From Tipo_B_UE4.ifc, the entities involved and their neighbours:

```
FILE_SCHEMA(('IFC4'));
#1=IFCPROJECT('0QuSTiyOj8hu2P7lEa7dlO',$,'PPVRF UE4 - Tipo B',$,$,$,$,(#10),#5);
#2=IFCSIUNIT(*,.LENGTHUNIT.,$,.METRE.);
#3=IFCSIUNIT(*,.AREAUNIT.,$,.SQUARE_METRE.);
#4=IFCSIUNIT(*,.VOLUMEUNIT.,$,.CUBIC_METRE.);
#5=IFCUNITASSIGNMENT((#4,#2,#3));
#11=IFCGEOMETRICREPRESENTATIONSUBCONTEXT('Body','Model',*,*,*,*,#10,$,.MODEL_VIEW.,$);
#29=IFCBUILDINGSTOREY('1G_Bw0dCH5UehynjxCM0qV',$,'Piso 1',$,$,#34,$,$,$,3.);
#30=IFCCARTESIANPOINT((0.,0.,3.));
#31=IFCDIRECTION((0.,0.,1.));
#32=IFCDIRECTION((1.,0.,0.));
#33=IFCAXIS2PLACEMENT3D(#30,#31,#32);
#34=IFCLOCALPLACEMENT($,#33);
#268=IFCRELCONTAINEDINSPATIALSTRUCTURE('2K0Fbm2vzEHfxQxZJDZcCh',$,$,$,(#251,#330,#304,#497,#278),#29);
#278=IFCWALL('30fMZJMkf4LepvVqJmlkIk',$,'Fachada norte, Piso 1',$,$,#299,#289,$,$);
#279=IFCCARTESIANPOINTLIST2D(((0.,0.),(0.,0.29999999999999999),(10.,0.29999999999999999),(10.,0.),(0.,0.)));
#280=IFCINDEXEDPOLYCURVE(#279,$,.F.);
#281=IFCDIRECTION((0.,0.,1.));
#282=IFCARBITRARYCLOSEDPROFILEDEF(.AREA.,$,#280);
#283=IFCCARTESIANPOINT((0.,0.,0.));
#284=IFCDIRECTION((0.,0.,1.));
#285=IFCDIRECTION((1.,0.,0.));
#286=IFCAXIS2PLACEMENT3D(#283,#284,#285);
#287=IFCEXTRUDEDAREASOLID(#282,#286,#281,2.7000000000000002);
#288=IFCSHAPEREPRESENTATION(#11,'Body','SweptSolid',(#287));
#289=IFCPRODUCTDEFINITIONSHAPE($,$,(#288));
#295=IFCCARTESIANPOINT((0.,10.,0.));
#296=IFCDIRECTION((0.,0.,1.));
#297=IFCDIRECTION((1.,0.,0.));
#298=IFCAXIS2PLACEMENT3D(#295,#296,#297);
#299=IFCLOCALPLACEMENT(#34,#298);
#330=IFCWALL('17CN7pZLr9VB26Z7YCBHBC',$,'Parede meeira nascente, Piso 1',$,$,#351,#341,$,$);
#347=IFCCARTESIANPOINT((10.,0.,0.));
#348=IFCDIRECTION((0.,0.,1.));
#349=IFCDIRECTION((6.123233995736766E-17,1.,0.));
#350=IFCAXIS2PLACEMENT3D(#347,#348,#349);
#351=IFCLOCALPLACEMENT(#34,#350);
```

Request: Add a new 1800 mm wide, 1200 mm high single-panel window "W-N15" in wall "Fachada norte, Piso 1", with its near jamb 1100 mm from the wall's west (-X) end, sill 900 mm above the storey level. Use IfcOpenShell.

```python
import numpy as np
import ifcopenshell
import ifcopenshell.api.feature
import ifcopenshell.api.geometry
import ifcopenshell.api.root
import ifcopenshell.api.spatial
import ifcopenshell.geom
import ifcopenshell.util.element
import ifcopenshell.util.placement
import ifcopenshell.util.representation
import ifcopenshell.util.shape
import ifcopenshell.util.unit

model = ifcopenshell.open("Tipo_B_UE4.ifc")
unit_scale = ifcopenshell.util.unit.calculate_unit_scale(model)
settings = ifcopenshell.geom.settings()


def volume(element):
    """Net volume in cubic metres, openings subtracted."""
    shape = ifcopenshell.geom.create_shape(settings, element)
    return ifcopenshell.util.shape.get_volume(shape.geometry)


wall = model.by_id(278)
storey = ifcopenshell.util.element.get_container(wall, ifc_class="IfcBuildingStorey")
context = ifcopenshell.util.representation.get_context(model, "Model", "Body", "MODEL_VIEW")
before = volume(wall)

width, height, from_end, sill = 1.8, 1.2, 1.1, 0.9  # metres

# The wall runs along its own X axis, and the end named is its -X end.
wall_shape = ifcopenshell.geom.create_shape(settings, wall)
x, y, z = ifcopenshell.util.shape.get_vertices(wall_shape.geometry).T
start = x.min() + from_end
face, thickness = float(y.min()), float(y.max() - y.min())
wall_matrix = ifcopenshell.util.placement.get_local_placement(wall.ObjectPlacement)
level = ifcopenshell.util.placement.get_local_placement(storey.ObjectPlacement)[2, 3]


def in_wall(x, y):
    """Placement at x, y metres in the wall's axes, at sill height."""
    matrix = wall_matrix.copy()
    matrix[:, 3] = wall_matrix @ np.array([x / unit_scale, y / unit_scale, 0.0, 1.0])
    matrix[2, 3] = level + sill / unit_scale
    return matrix


# Opening: a box that overshoots both wall faces by 50 mm.
opening = ifcopenshell.api.root.create_entity(model, ifc_class="IfcOpeningElement", predefined_type="OPENING")
box = ifcopenshell.api.geometry.add_wall_representation(
    model, context=context, length=width, height=height, thickness=thickness + 0.1
)
ifcopenshell.api.geometry.assign_representation(model, product=opening, representation=box)
ifcopenshell.api.geometry.edit_object_placement(model, product=opening, matrix=in_wall(start, face - 0.05), is_si=False)
ifcopenshell.api.feature.add_feature(model, feature=opening, element=wall)

window = ifcopenshell.api.root.create_entity(model, ifc_class="IfcWindow", name="W-N15", predefined_type="WINDOW")
window.OverallWidth, window.OverallHeight = width / unit_scale, height / unit_scale
window.PartitioningType = "SINGLE_PANEL"
body = ifcopenshell.api.geometry.add_window_representation(
    model,
    context=context,
    overall_width=window.OverallWidth,
    overall_height=window.OverallHeight,
    partition_type="SINGLE_PANEL",
)
ifcopenshell.api.geometry.assign_representation(model, product=window, representation=body)
ifcopenshell.api.spatial.assign_container(model, products=[window], relating_structure=storey)
ifcopenshell.api.feature.add_filling(model, opening=opening, element=window)

# Centre the window in the wall's thickness.
ifcopenshell.api.geometry.edit_object_placement(model, product=window, matrix=in_wall(start, face), is_si=False)
window_shape = ifcopenshell.geom.create_shape(settings, window)
depth = ifcopenshell.util.shape.get_vertices(window_shape.geometry)[:, 1]
offset = face + thickness / 2 - (depth.min() + depth.max()) / 2
ifcopenshell.api.geometry.edit_object_placement(model, product=window, matrix=in_wall(start, offset), is_si=False)

after = volume(wall)

print(f"wall volume {before:.3f} -> {after:.3f} m3")

model.write("Tipo_B_UE4_edited.ifc")
```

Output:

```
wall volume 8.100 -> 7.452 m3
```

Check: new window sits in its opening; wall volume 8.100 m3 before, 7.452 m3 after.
